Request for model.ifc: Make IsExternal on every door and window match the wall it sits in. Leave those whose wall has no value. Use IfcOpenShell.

First a look at what the model holds.

```python
import ifcopenshell
import ifcopenshell.util.element

model = ifcopenshell.open("model.ifc")
print(model.schema)
seen = {}
for e in model.by_type("IfcDoor") + model.by_type("IfcWindow"):
    if not e.FillsVoids:
        continue
    host = e.FillsVoids[0].RelatingOpeningElement.VoidsElements[0].RelatingBuildingElement
    own = ifcopenshell.util.element.get_pset(e, f"Pset_{e.is_a()[3:].removesuffix('StandardCase')}Common", "IsExternal")
    wall = ifcopenshell.util.element.get_pset(host, "Pset_WallCommon", "IsExternal")
    seen[e.is_a(), own, wall] = seen.get((e.is_a(), own, wall), 0) + 1
for (cls, own, wall), count in sorted(seen.items(), key=str):
    print(count, cls, "IsExternal:", own, "| host wall:", wall)
```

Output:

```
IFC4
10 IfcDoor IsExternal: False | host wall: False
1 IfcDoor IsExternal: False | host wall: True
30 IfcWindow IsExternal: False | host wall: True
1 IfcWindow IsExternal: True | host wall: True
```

```python
import ifcopenshell
import ifcopenshell.api.pset
import ifcopenshell.util.element

model = ifcopenshell.open("model.ifc")

count = 0
for ifc_class, pset_name in (("IfcDoor", "Pset_DoorCommon"), ("IfcWindow", "Pset_WindowCommon")):
    for e in model.by_type(ifc_class):
        if not e.FillsVoids:
            continue
        host = e.FillsVoids[0].RelatingOpeningElement.VoidsElements[0].RelatingBuildingElement
        external = ifcopenshell.util.element.get_pset(host, "Pset_WallCommon", "IsExternal")
        if external is None or ifcopenshell.util.element.get_pset(e, pset_name, "IsExternal") == external:
            continue
        pset = ifcopenshell.api.pset.add_pset(model, product=e, name=pset_name)
        ifcopenshell.api.pset.edit_pset(model, pset=pset, properties={"IsExternal": external})
        count += 1

print(count, "updated")

model.write("model-out.ifc")
```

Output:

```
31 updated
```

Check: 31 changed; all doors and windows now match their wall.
